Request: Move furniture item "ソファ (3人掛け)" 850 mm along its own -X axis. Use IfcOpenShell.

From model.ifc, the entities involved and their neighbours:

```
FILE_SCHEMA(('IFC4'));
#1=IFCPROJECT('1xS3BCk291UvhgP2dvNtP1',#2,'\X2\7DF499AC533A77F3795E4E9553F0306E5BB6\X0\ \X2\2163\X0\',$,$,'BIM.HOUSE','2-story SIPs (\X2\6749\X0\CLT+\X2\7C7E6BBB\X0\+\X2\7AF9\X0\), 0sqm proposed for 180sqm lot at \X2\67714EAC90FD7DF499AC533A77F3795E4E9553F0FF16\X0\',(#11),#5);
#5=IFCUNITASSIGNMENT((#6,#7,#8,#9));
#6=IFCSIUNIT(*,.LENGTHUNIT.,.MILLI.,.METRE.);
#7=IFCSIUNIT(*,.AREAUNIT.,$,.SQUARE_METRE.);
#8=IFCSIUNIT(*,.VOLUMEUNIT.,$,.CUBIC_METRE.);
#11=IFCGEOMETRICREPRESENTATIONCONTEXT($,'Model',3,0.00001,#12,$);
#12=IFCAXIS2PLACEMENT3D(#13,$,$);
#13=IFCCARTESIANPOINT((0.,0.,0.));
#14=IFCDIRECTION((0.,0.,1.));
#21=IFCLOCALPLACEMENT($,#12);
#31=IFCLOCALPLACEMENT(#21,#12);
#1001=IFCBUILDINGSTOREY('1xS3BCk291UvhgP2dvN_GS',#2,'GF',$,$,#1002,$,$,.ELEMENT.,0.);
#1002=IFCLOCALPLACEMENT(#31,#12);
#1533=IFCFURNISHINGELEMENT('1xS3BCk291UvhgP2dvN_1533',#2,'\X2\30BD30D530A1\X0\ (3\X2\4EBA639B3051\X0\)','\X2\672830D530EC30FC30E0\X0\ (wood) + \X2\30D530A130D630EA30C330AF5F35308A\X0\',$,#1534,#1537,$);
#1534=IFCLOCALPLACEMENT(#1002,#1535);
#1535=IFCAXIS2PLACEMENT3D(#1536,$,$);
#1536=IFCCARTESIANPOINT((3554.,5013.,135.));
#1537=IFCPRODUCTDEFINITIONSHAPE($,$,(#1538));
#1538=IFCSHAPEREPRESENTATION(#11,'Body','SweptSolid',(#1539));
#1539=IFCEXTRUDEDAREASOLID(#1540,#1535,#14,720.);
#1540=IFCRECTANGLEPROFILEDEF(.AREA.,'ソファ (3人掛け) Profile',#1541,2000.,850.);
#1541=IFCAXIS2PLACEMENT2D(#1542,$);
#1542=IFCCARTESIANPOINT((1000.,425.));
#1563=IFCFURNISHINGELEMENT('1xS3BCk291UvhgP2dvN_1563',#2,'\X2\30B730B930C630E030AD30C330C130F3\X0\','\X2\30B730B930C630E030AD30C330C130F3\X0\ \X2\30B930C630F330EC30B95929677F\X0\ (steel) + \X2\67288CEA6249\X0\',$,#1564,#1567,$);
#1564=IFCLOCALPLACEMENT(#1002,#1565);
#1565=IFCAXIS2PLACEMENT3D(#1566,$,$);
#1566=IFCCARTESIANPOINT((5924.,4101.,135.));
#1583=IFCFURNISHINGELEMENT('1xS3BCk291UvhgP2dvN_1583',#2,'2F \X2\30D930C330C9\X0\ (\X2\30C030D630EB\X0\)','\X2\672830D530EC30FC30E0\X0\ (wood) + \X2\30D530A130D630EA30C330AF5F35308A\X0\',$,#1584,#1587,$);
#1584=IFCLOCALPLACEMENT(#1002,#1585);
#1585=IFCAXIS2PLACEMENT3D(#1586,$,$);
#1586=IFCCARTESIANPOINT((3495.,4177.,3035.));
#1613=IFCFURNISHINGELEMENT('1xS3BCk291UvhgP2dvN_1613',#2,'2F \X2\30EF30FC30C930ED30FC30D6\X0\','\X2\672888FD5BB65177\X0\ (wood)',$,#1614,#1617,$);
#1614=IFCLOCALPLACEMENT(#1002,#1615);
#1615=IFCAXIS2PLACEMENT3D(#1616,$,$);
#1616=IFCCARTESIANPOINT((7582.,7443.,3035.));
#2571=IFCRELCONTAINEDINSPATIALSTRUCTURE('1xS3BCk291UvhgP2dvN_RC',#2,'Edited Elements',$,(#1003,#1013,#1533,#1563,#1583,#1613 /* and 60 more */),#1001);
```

```python
import ifcopenshell
import ifcopenshell.api.geometry
import ifcopenshell.util.placement
import ifcopenshell.util.unit

model = ifcopenshell.open("model.ifc")
unit_scale = ifcopenshell.util.unit.calculate_unit_scale(model)

item = model.by_guid("1xS3BCk291UvhgP2dvN_1533")
matrix = ifcopenshell.util.placement.get_local_placement(item.ObjectPlacement)
matrix[:3, 3] -= matrix[:3, 0] * 0.85 / unit_scale
ifcopenshell.api.geometry.edit_object_placement(model, product=item, matrix=matrix, is_si=False)

print(ifcopenshell.util.placement.get_local_placement(item.ObjectPlacement).round(3) + 0.0)

model.write("model-out.ifc")
```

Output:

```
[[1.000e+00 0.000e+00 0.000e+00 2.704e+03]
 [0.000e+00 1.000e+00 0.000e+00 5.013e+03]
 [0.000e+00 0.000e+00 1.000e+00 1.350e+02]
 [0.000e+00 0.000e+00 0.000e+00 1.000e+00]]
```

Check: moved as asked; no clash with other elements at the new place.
